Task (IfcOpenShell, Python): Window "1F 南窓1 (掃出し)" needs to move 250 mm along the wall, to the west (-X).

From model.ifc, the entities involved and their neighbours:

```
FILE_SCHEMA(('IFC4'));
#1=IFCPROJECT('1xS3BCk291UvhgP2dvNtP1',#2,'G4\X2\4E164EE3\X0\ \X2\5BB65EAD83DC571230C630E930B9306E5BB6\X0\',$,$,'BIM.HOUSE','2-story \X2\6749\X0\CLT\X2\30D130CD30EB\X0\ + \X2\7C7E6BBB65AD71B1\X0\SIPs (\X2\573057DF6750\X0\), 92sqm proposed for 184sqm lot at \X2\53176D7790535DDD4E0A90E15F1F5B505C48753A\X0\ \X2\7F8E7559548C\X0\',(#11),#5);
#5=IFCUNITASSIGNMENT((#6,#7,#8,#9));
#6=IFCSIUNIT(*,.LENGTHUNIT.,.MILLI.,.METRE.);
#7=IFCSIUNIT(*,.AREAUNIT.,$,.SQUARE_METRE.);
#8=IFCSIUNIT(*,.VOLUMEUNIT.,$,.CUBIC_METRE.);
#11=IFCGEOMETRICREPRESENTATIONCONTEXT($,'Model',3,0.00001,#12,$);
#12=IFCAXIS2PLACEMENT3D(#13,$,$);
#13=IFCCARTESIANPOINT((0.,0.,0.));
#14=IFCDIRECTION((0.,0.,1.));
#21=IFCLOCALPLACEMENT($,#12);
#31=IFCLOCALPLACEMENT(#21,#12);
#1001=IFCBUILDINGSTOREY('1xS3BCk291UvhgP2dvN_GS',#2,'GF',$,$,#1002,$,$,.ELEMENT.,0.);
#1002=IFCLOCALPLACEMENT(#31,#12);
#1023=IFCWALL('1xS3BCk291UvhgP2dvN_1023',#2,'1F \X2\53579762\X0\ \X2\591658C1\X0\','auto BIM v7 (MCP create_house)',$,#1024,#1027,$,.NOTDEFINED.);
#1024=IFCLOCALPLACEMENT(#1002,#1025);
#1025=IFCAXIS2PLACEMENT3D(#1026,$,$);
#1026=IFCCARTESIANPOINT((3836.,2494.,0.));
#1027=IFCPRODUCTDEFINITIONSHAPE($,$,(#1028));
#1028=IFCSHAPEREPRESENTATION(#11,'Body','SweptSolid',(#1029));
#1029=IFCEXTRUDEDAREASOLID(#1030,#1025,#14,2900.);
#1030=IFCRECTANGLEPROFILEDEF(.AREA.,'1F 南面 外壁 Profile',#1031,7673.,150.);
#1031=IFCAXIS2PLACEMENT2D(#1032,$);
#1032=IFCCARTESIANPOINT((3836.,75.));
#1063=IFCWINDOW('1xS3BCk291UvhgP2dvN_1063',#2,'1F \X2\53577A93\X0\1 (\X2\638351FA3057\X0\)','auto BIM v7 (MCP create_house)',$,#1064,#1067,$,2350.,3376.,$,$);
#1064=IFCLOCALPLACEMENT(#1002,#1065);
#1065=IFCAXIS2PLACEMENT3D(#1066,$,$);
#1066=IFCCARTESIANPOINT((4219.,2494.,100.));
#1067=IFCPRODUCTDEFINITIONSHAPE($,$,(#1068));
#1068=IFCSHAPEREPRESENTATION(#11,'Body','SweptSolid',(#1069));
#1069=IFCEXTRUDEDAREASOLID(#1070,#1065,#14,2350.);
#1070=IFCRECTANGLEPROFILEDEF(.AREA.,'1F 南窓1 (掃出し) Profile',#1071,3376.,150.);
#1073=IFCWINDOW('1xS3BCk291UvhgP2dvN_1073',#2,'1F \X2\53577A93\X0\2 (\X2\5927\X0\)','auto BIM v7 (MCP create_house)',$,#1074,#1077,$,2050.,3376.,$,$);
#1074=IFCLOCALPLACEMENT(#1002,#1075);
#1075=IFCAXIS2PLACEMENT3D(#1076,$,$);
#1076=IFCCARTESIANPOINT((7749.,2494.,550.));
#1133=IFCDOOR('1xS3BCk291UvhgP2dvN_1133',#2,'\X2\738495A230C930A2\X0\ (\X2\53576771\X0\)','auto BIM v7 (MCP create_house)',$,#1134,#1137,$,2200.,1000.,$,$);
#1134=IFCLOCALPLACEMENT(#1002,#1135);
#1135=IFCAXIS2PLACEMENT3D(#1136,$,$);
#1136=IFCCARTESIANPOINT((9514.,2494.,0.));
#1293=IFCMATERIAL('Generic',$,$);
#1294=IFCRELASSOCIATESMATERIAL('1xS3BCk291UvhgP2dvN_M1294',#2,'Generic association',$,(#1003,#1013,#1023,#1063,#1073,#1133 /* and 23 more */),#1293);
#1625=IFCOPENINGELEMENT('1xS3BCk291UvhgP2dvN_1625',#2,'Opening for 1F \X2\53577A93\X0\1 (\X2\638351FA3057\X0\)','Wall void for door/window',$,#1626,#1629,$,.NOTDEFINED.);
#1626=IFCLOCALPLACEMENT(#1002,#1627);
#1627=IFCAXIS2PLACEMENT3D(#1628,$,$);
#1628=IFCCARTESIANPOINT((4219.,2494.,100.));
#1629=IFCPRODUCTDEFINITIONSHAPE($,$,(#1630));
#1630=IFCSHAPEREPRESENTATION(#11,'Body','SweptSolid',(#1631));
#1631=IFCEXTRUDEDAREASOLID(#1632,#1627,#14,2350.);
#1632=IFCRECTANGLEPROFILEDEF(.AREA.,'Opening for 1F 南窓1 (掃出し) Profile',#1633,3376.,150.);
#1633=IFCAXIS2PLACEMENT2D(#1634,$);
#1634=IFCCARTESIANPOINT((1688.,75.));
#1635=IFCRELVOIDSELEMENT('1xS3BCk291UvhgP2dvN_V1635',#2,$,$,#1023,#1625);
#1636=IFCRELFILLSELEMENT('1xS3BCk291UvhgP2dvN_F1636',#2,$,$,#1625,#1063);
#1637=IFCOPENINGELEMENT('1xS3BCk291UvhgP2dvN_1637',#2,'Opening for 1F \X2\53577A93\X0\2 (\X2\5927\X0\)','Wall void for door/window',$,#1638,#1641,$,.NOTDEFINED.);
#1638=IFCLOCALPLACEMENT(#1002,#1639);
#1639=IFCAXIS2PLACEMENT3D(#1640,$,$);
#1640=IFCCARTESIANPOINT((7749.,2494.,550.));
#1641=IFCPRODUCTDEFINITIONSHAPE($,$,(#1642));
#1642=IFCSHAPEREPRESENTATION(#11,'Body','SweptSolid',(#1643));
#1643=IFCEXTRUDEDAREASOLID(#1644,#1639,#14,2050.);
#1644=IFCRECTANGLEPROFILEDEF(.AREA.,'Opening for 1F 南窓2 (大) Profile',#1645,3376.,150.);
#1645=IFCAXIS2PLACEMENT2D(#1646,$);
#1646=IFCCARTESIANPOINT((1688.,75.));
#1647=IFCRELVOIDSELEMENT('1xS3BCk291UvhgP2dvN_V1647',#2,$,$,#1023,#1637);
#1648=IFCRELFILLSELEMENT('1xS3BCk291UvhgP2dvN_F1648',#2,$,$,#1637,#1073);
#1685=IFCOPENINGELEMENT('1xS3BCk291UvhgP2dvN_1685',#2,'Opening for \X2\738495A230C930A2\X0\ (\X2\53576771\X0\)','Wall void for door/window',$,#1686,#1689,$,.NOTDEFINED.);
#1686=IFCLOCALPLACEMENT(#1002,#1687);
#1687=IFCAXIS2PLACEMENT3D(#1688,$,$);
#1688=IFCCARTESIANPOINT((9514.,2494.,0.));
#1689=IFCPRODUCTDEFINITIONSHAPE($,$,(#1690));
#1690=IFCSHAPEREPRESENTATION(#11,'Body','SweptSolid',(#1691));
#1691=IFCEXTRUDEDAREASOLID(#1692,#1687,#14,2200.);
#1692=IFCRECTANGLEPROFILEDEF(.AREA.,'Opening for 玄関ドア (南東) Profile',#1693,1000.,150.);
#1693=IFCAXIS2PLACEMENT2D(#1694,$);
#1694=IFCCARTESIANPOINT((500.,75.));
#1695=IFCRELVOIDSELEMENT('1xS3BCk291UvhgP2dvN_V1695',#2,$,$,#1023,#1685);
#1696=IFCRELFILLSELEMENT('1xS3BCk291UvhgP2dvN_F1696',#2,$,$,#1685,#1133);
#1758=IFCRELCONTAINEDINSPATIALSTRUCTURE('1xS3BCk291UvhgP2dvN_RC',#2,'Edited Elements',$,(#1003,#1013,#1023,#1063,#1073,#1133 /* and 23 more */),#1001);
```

```python
import ifcopenshell
import ifcopenshell.api.geometry
import ifcopenshell.util.placement
import ifcopenshell.util.unit

model = ifcopenshell.open("model.ifc")
unit_scale = ifcopenshell.util.unit.calculate_unit_scale(model)

window = model.by_guid("1xS3BCk291UvhgP2dvN_1063")
opening = window.FillsVoids[0].RelatingOpeningElement
wall = opening.VoidsElements[0].RelatingBuildingElement

wall_matrix = ifcopenshell.util.placement.get_local_placement(wall.ObjectPlacement)
shift = wall_matrix[:3, 0] * -0.25 / unit_scale
before = ifcopenshell.util.placement.get_local_placement(window.ObjectPlacement)[:3, 3].copy()

# The window is not placed relative to its opening, so move both.
for product in (opening, window):
    matrix = ifcopenshell.util.placement.get_local_placement(product.ObjectPlacement)
    matrix[:3, 3] += shift
    ifcopenshell.api.geometry.edit_object_placement(model, product=product, matrix=matrix, is_si=False)

after = ifcopenshell.util.placement.get_local_placement(window.ObjectPlacement)[:3, 3]
print("window moved by", (after - before).round(3) + 0.0)

model.write("model_updated.ifc")
```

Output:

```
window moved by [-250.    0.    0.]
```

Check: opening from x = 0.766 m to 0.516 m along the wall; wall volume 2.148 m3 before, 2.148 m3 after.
